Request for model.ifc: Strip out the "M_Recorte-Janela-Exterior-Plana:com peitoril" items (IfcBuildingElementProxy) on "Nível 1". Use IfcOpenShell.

First a look at what the model holds.

```python
import ifcopenshell
import ifcopenshell.util.element

model = ifcopenshell.open("model.ifc")
print(model.schema)
storey = next(s for s in model.by_type("IfcBuildingStorey") if s.Name == "Nível 1")
proxies = [e for e in ifcopenshell.util.element.get_decomposition(storey) if e.is_a("IfcBuildingElementProxy")]
seen = {}
for e in proxies:
    element_type = ifcopenshell.util.element.get_type(e)
    name = element_type.Name if element_type not in (None, e) else None
    seen[name] = seen.get(name, 0) + 1
for name, count in sorted(seen.items(), key=str):
    print(count, "x", name)
```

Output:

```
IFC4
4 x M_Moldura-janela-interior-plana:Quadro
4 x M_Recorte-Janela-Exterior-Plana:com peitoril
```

```python
import ifcopenshell
import ifcopenshell.api.root
import ifcopenshell.util.element

model = ifcopenshell.open("model.ifc")

storey = next(s for s in model.by_type("IfcBuildingStorey") if s.Name == "Nível 1")
proxies = [e for e in ifcopenshell.util.element.get_decomposition(storey) if e.is_a("IfcBuildingElementProxy")]
targets = [e for e in proxies if (t := ifcopenshell.util.element.get_type(e)) not in (None, e) and t.Name == "M_Recorte-Janela-Exterior-Plana:com peitoril"]

for e in targets:
    ifcopenshell.api.root.remove_product(model, product=e)
print(len(targets), "removed")

model.write("model_edited.ifc")
```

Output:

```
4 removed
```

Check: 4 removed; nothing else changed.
